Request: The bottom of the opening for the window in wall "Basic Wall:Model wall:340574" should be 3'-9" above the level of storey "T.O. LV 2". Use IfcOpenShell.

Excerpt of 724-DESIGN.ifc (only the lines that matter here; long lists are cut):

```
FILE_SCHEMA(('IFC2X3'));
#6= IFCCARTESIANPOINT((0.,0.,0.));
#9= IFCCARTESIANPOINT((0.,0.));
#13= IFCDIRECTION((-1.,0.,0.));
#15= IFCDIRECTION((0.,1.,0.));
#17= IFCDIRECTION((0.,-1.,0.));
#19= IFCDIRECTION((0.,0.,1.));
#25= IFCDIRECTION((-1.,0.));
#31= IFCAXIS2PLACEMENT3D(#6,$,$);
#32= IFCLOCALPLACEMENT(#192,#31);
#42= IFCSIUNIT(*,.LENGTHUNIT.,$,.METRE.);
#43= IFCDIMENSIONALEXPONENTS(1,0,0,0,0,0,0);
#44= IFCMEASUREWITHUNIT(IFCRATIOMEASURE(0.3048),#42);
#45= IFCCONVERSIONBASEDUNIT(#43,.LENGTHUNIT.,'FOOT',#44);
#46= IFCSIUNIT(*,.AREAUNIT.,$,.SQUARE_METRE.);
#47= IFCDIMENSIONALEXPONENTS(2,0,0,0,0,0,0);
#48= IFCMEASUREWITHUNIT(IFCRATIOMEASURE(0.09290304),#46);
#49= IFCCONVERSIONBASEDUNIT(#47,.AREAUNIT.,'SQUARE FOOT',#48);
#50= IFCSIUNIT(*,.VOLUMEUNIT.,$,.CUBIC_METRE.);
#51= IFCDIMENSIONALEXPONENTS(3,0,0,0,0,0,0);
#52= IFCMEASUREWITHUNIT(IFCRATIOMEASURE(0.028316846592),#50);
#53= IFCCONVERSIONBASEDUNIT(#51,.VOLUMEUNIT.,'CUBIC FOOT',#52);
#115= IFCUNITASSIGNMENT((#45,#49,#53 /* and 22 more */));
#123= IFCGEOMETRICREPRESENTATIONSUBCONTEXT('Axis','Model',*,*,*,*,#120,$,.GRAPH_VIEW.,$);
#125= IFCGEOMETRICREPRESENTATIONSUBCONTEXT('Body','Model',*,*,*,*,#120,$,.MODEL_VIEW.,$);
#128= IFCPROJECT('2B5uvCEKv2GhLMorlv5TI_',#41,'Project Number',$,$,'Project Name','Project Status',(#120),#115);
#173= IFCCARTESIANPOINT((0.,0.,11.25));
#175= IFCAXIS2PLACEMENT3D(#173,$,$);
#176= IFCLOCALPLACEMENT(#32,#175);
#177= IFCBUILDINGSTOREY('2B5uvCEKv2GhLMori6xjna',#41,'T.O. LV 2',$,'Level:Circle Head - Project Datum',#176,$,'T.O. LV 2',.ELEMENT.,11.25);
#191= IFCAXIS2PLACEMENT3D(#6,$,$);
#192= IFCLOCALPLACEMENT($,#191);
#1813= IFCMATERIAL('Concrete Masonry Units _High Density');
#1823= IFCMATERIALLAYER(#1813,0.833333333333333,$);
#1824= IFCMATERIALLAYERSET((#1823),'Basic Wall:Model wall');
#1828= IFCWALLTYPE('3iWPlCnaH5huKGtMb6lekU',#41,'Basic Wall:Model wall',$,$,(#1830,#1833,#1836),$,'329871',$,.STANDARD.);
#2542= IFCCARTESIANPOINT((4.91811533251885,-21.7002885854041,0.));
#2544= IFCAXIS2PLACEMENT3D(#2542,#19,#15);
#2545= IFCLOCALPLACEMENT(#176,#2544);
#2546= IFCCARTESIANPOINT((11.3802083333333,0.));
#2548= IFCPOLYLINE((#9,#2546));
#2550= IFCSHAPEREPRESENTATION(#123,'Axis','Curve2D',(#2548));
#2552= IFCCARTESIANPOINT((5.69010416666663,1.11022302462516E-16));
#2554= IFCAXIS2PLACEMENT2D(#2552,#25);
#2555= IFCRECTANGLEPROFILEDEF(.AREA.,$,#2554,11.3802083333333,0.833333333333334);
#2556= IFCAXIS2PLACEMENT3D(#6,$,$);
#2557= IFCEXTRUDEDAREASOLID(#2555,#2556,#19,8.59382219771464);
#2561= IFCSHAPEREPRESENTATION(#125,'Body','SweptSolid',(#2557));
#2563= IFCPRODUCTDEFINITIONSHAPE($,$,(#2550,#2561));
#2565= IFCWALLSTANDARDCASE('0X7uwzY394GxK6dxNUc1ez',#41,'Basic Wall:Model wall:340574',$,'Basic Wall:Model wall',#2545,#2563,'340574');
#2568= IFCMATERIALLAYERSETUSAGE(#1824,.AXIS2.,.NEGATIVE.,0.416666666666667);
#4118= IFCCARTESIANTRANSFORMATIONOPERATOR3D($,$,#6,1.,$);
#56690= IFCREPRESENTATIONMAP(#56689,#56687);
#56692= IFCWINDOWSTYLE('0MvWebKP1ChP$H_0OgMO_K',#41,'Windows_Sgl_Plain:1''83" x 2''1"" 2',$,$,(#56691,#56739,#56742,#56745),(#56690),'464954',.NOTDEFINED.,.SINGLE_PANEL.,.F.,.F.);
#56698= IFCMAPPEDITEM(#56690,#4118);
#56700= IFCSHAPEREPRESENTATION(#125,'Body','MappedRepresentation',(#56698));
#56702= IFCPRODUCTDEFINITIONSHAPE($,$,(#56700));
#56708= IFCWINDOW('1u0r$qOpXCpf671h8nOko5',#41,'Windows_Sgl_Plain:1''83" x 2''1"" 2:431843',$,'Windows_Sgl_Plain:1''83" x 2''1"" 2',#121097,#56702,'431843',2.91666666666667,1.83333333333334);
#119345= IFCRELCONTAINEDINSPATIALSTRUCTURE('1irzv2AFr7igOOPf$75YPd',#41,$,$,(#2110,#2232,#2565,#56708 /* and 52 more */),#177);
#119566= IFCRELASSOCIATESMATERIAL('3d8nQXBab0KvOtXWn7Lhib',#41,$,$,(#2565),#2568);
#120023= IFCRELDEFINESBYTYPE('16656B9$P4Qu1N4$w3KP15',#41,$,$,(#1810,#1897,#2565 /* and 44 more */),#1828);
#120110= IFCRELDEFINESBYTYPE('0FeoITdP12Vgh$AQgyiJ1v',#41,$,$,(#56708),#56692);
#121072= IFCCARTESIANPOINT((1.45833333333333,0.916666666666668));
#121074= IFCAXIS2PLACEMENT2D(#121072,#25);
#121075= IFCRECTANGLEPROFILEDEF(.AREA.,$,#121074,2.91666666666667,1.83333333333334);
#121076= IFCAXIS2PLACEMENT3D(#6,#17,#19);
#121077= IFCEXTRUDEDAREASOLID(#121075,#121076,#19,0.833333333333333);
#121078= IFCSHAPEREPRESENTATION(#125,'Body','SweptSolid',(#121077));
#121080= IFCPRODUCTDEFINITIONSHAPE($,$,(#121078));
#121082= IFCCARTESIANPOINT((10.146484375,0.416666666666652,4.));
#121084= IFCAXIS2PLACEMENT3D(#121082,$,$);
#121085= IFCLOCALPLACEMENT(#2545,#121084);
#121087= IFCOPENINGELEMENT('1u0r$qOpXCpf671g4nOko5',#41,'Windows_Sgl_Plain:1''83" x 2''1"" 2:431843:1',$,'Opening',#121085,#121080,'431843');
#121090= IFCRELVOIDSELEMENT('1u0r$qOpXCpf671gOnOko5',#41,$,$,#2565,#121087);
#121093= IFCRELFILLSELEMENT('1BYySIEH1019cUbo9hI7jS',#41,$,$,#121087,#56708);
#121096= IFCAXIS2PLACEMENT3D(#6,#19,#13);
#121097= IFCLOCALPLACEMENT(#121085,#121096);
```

```python
import numpy as np
import ifcopenshell
import ifcopenshell.api.geometry
import ifcopenshell.geom
import ifcopenshell.util.element
import ifcopenshell.util.placement
import ifcopenshell.util.shape
import ifcopenshell.util.unit

model = ifcopenshell.open("724-DESIGN.ifc")
unit_scale = ifcopenshell.util.unit.calculate_unit_scale(model)

window = model.by_guid("1u0r$qOpXCpf671h8nOko5")
opening = window.FillsVoids[0].RelatingOpeningElement
storey = ifcopenshell.util.element.get_container(window, ifc_class="IfcBuildingStorey")
level = ifcopenshell.util.placement.get_local_placement(storey.ObjectPlacement)[2, 3]

# The opening's origin need not be at the sill, so measure its lowest point.
shape = ifcopenshell.geom.create_shape(ifcopenshell.geom.settings(), opening)
bottom = ifcopenshell.util.shape.get_shape_bottom_elevation(shape, shape.geometry) / unit_scale
dz = level + 45 * 0.0254 / unit_scale - bottom

shift = np.array([0.0, 0.0, dz])
# The window is placed relative to its opening, so it follows when the opening moves.
matrix = ifcopenshell.util.placement.get_local_placement(opening.ObjectPlacement)
matrix[:3, 3] += shift
ifcopenshell.api.geometry.edit_object_placement(
    model, product=opening, matrix=matrix, is_si=False, should_transform_children=True
)

print(f"moved by {dz * unit_scale:+.3f} m")

model.write("724-DESIGN_updated.ifc")
```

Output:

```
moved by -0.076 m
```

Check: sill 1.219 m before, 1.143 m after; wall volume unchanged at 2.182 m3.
